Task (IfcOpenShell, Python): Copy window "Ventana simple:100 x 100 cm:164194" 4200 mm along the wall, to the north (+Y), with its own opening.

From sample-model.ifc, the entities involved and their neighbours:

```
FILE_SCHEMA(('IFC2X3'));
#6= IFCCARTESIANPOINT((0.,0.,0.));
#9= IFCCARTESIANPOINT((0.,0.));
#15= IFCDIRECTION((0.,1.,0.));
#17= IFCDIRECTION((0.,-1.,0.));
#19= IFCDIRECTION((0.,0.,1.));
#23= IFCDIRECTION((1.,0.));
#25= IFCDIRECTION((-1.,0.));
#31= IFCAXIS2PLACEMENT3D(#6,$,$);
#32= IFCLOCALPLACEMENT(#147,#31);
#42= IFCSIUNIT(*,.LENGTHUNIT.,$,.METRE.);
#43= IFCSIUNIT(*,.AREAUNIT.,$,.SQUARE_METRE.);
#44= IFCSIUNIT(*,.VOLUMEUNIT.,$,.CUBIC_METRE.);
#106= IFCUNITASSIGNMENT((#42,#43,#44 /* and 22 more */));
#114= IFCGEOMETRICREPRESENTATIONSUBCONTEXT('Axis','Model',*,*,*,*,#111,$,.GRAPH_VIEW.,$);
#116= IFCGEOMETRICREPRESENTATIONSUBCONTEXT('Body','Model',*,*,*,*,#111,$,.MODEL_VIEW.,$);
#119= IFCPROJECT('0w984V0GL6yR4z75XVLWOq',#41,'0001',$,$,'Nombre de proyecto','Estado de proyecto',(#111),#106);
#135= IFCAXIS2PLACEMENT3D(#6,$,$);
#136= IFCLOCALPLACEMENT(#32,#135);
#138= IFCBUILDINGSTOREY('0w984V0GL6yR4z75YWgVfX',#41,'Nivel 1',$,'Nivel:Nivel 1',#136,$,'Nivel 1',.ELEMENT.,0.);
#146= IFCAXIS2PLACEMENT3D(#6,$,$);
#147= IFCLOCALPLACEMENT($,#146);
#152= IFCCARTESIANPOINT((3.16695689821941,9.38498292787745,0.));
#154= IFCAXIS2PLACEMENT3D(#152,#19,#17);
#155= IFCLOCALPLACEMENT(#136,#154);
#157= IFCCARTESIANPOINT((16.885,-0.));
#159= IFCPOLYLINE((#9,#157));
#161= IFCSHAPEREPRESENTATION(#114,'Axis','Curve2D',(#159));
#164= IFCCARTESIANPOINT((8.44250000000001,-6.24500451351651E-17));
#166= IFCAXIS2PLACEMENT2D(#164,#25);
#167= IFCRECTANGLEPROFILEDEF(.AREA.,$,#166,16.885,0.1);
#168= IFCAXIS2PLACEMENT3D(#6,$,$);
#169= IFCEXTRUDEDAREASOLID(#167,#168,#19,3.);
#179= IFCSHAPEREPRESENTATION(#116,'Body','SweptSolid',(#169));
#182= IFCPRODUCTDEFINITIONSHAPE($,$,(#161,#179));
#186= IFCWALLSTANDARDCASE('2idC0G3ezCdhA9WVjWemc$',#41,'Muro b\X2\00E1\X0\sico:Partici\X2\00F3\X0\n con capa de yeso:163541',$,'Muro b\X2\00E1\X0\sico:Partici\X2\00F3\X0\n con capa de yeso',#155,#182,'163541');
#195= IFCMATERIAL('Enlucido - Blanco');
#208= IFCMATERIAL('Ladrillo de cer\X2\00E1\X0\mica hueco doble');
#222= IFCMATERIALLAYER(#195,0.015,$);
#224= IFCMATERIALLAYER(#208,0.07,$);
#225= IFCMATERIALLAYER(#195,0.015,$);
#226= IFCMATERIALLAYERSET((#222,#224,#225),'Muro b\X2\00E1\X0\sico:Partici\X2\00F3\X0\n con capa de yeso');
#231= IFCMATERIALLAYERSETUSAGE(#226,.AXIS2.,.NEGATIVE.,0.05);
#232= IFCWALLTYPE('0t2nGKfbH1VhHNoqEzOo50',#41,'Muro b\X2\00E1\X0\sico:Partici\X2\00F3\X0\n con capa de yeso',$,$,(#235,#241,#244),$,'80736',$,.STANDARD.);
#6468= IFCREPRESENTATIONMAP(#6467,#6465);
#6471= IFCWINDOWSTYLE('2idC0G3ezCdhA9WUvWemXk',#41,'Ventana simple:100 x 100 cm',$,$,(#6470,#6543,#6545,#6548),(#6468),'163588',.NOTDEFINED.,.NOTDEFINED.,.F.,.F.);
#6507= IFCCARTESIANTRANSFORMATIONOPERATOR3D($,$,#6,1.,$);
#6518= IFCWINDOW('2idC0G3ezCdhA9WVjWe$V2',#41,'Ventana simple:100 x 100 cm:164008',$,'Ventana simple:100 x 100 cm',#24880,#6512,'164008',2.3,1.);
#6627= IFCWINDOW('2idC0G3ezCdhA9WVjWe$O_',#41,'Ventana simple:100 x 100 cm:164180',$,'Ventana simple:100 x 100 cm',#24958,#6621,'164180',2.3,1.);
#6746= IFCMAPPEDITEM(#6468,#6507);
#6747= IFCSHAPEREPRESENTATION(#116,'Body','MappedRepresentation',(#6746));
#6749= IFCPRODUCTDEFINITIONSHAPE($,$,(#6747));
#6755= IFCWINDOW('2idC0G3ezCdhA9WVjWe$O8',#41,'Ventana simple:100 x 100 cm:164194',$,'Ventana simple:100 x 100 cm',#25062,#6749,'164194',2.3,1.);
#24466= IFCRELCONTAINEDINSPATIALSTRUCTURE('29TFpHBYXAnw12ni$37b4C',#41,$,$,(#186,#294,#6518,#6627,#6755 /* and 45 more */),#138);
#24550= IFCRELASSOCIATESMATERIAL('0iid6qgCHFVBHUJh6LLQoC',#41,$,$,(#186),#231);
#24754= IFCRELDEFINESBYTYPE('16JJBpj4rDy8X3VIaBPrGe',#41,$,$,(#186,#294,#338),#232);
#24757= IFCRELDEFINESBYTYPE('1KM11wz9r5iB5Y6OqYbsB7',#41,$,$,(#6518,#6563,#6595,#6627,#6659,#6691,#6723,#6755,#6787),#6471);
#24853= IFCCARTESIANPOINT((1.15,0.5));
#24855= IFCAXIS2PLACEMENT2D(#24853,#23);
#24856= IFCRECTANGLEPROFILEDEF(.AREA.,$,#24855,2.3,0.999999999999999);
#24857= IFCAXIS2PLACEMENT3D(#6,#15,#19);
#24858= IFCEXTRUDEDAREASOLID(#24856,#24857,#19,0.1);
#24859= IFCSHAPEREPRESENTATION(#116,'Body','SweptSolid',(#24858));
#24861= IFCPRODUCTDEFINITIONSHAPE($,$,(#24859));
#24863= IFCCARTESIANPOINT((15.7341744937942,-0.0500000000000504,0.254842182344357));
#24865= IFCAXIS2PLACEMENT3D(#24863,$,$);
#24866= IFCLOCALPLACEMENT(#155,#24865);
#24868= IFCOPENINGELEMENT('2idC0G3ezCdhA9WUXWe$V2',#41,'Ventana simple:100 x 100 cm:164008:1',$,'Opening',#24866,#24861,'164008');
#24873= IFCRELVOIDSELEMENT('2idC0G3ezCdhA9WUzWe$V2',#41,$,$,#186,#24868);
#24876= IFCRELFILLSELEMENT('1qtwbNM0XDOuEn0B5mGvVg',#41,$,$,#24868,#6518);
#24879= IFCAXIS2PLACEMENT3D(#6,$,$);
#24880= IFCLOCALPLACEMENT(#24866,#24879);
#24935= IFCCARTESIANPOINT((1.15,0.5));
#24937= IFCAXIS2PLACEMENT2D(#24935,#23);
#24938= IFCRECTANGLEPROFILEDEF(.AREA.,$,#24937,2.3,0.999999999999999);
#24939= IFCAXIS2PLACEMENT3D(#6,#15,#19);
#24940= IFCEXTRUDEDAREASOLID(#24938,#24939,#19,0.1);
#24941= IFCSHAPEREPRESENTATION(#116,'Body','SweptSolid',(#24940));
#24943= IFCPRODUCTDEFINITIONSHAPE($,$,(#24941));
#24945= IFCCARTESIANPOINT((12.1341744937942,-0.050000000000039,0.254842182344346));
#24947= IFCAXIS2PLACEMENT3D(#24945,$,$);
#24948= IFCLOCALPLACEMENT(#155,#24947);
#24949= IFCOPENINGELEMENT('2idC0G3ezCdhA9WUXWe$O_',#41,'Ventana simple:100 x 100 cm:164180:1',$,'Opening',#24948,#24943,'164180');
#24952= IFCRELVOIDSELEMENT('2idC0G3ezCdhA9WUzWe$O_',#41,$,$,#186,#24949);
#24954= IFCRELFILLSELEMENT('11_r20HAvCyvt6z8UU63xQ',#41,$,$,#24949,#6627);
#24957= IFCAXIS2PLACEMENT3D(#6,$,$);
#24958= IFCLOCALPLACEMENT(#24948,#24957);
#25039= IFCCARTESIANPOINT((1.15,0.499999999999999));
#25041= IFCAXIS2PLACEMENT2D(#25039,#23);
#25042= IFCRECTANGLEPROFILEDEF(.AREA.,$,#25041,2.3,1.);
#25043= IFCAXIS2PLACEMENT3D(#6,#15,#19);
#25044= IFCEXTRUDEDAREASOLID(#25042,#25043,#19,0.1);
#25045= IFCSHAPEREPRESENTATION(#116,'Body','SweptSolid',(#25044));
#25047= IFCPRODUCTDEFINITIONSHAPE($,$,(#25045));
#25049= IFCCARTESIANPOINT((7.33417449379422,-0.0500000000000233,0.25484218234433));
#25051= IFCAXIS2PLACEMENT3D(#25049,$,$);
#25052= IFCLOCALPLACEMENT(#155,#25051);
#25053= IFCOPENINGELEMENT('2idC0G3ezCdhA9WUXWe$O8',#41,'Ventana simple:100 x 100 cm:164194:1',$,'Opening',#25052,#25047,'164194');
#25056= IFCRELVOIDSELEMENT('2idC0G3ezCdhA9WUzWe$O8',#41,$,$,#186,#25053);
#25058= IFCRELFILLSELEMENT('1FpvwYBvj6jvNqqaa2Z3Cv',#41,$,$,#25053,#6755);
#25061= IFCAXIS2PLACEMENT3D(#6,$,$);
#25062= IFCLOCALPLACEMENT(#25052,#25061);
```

```python
import ifcopenshell
import ifcopenshell.api.feature
import ifcopenshell.api.geometry
import ifcopenshell.api.root
import ifcopenshell.geom
import ifcopenshell.util.element
import ifcopenshell.util.placement
import ifcopenshell.util.shape

model = ifcopenshell.open("sample-model.ifc")
settings = ifcopenshell.geom.settings()


def volume(element):
    """Net volume in cubic metres, openings subtracted."""
    shape = ifcopenshell.geom.create_shape(settings, element)
    return ifcopenshell.util.shape.get_volume(shape.geometry)


def reuse_history(source, copy):
    """copy_class also copies each property set's owner history, people and application; keep the originals."""
    for rel in copy.IsDefinedBy:
        if rel.is_a("IfcRelDefinesByProperties") and (history := rel.RelatingPropertyDefinition.OwnerHistory):
            rel.RelatingPropertyDefinition.OwnerHistory = source.OwnerHistory
            ifcopenshell.util.element.remove_deep2(model, history)


window = model.by_id(6755)
opening = window.FillsVoids[0].RelatingOpeningElement
wall = opening.VoidsElements[0].RelatingBuildingElement
before = volume(wall)
shift = ifcopenshell.util.placement.get_local_placement(wall.ObjectPlacement)[:3, 0] * -4.2

# copy_class copies the void relationship, type, container and properties, but no geometry.
new_opening = ifcopenshell.api.root.copy_class(model, product=opening)
new_opening.Representation = ifcopenshell.util.element.copy_deep(
    model, opening.Representation, exclude=["IfcGeometricRepresentationContext", "IfcRepresentationMap"]
)
new_opening.Name = "Ventana simple:100 x 100 cm"
new_opening.Tag = None
new_window = ifcopenshell.api.root.copy_class(model, product=window)
new_window.Representation = ifcopenshell.util.element.copy_deep(
    model, window.Representation, exclude=["IfcGeometricRepresentationContext", "IfcRepresentationMap"]
)
new_window.Name = "Ventana simple:100 x 100 cm"
new_window.Tag = None
reuse_history(window, new_window)
fills = ifcopenshell.api.feature.add_filling(model, opening=new_opening, element=new_window)
fills.OwnerHistory = new_window.OwnerHistory  # required in IFC2X3

for old, new in ((opening, new_opening), (window, new_window)):
    matrix = ifcopenshell.util.placement.get_local_placement(old.ObjectPlacement)
    matrix[:3, 3] += shift
    ifcopenshell.api.geometry.edit_object_placement(model, product=new, matrix=matrix, is_si=False)

after = volume(wall)

print(f"wall volume {before:.3f} -> {after:.3f} m3")

model.write("sample-model_rev.ifc")
```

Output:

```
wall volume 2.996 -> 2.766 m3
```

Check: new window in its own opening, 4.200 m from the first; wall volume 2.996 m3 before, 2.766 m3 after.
